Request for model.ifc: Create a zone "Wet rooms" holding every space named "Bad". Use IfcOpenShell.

First a look at what the model holds.

```python
import ifcopenshell

model = ifcopenshell.open("model.ifc")
print(model.schema)
seen = {}
for space in model.by_type("IfcSpace"):
    seen[space.LongName] = seen.get(space.LongName, 0) + 1
for name, count in sorted(seen.items(), key=str):
    print(count, "x", name)
print("zones:", [z.Name for z in model.by_type("IfcZone")][:20])
```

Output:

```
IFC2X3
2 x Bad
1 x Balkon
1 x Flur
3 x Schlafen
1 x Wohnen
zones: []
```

```python
import ifcopenshell
import ifcopenshell.api.group
import ifcopenshell.api.root

model = ifcopenshell.open("model.ifc")

names = {"Bad"}
spaces = [s for s in model.by_type("IfcSpace") if s.LongName in names]

zone = ifcopenshell.api.root.create_entity(model, ifc_class="IfcZone", name="Wet rooms")
ifcopenshell.api.group.assign_group(model, products=spaces, group=zone)
print(len(spaces), "spaces in", zone.Name)

model.write("model_updated.ifc")
```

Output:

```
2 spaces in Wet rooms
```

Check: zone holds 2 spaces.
